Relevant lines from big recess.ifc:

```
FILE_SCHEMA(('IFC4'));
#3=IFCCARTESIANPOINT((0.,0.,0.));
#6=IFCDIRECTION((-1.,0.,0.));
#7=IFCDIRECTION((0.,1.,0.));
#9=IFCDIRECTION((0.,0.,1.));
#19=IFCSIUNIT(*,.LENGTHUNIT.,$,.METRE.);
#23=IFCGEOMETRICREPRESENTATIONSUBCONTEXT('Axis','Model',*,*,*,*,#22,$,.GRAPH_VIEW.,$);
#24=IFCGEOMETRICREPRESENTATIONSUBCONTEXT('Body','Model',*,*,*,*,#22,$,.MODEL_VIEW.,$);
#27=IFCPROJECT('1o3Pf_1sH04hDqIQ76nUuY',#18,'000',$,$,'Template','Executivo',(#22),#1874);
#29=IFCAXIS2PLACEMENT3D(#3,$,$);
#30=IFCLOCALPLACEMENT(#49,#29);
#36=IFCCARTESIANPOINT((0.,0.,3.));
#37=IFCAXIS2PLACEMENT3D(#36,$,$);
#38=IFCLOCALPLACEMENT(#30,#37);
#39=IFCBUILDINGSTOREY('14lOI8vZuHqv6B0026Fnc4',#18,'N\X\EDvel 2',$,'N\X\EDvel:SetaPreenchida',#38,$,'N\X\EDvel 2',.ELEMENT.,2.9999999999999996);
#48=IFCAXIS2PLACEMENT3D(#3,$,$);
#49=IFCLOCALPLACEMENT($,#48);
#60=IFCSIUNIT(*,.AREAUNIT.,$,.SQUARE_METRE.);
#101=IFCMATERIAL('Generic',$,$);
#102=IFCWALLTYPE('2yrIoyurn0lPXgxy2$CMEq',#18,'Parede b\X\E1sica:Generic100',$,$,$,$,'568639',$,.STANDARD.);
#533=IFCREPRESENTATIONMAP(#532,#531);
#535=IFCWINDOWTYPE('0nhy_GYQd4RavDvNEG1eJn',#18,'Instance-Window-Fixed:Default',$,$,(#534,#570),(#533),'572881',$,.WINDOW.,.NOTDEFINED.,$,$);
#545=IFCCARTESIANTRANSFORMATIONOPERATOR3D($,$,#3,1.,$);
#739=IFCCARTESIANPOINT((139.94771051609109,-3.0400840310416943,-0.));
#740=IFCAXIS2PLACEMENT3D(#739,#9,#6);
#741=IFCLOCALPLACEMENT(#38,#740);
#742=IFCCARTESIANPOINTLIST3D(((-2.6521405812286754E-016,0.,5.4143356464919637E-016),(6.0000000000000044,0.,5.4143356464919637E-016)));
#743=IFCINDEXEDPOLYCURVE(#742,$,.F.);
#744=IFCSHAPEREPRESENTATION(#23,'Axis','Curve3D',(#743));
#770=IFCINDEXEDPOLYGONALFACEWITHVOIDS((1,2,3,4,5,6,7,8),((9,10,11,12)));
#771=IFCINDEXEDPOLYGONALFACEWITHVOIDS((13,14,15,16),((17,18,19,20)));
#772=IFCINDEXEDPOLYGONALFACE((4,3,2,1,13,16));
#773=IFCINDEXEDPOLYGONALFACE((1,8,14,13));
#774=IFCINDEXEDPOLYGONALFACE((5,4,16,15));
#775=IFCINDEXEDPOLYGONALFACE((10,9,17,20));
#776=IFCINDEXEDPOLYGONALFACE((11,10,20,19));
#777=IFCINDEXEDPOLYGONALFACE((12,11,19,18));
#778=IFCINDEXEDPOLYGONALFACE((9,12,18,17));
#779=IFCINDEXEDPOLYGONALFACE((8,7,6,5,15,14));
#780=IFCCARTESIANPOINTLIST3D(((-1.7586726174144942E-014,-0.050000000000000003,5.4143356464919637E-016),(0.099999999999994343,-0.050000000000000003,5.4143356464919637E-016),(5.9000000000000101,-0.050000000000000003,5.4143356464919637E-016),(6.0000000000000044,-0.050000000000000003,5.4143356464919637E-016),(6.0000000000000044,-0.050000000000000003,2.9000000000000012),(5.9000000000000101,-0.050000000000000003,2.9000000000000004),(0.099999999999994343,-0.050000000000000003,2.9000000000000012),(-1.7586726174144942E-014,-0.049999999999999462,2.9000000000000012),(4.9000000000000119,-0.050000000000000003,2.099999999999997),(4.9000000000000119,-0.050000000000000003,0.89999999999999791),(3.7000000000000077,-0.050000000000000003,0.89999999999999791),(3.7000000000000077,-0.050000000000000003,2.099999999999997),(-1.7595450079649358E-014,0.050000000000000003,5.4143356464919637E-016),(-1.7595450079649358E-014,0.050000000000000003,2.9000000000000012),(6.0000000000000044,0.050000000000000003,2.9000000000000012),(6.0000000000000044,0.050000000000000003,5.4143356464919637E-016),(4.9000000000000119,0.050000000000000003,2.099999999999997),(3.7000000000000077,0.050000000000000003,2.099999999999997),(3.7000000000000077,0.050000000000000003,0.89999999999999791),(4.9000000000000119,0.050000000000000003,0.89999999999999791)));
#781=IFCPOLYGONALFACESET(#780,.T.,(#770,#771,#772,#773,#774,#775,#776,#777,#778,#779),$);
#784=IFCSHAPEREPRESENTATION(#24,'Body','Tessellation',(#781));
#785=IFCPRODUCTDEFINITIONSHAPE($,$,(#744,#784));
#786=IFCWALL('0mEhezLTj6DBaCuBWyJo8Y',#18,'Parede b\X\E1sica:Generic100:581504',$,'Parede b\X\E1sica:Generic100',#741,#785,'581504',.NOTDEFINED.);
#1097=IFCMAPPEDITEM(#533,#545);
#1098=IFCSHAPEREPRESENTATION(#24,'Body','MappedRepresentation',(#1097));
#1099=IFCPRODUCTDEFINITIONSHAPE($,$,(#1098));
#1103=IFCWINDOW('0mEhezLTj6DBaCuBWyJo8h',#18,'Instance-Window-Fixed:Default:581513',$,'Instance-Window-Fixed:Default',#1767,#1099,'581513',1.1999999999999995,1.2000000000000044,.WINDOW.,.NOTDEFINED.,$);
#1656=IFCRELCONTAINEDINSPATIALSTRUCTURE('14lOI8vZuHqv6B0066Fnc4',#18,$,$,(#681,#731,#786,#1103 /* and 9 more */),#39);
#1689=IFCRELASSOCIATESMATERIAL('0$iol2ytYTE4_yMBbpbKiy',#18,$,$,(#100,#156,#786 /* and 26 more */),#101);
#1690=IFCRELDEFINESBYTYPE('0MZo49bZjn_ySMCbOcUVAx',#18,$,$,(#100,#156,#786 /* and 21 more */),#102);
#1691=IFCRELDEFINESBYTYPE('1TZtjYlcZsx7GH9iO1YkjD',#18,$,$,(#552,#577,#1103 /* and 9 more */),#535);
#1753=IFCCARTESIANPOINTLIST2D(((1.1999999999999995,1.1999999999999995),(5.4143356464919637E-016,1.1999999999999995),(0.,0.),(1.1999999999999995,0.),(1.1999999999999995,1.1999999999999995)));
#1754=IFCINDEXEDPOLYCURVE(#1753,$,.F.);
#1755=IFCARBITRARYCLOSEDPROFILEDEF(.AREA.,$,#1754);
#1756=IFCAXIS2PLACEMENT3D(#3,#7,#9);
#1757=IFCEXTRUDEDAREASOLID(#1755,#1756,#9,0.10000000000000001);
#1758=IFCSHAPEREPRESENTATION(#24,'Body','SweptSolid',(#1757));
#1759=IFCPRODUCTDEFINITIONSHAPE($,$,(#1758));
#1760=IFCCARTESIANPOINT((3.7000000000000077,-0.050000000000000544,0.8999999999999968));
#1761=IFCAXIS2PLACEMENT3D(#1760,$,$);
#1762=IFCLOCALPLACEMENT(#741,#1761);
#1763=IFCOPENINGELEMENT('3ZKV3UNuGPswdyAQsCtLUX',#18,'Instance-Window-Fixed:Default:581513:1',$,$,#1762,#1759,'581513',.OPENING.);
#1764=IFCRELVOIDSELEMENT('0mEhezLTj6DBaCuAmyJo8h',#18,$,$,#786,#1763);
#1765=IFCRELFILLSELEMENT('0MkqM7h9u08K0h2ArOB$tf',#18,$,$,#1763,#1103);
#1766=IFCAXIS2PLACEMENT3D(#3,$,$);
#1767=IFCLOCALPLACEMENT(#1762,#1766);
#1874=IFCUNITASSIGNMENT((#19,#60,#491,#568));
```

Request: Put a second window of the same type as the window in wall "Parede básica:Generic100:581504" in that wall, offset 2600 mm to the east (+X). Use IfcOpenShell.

```python
import ifcopenshell
import ifcopenshell.api.feature
import ifcopenshell.api.geometry
import ifcopenshell.api.root
import ifcopenshell.geom
import ifcopenshell.util.element
import ifcopenshell.util.placement
import ifcopenshell.util.shape

model = ifcopenshell.open("big recess.ifc")
settings = ifcopenshell.geom.settings()


def volume(element):
    """Net volume in cubic metres, openings subtracted."""
    shape = ifcopenshell.geom.create_shape(settings, element)
    return ifcopenshell.util.shape.get_volume(shape.geometry)


def reuse_history(source, copy):
    """copy_class also copies each property set's owner history, people and application; keep the originals."""
    for rel in copy.IsDefinedBy:
        if rel.is_a("IfcRelDefinesByProperties") and (history := rel.RelatingPropertyDefinition.OwnerHistory):
            rel.RelatingPropertyDefinition.OwnerHistory = source.OwnerHistory
            ifcopenshell.util.element.remove_deep2(model, history)


window = model.by_guid("0mEhezLTj6DBaCuBWyJo8h")
opening = window.FillsVoids[0].RelatingOpeningElement
wall = opening.VoidsElements[0].RelatingBuildingElement
before = volume(wall)
shift = ifcopenshell.util.placement.get_local_placement(wall.ObjectPlacement)[:3, 0] * -2.6

# copy_class copies the void relationship, type, container and properties, but no geometry.
new_opening = ifcopenshell.api.root.copy_class(model, product=opening)
new_opening.Representation = ifcopenshell.util.element.copy_deep(
    model, opening.Representation, exclude=["IfcGeometricRepresentationContext", "IfcRepresentationMap"]
)
new_opening.Name = "Instance-Window-Fixed:Default"
new_opening.Tag = None
new_window = ifcopenshell.api.root.copy_class(model, product=window)
new_window.Representation = ifcopenshell.util.element.copy_deep(
    model, window.Representation, exclude=["IfcGeometricRepresentationContext", "IfcRepresentationMap"]
)
new_window.Name = "Instance-Window-Fixed:Default"
new_window.Tag = None
reuse_history(window, new_window)
ifcopenshell.api.feature.add_filling(model, opening=new_opening, element=new_window)

for old, new in ((opening, new_opening), (window, new_window)):
    matrix = ifcopenshell.util.placement.get_local_placement(old.ObjectPlacement)
    matrix[:3, 3] += shift
    ifcopenshell.api.geometry.edit_object_placement(model, product=new, matrix=matrix, is_si=False)

after = volume(wall)

print(f"wall volume {before:.3f} -> {after:.3f} m3")

model.write("big recess-out.ifc")
```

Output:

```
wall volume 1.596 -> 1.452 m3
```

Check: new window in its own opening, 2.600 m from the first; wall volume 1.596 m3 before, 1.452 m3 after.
